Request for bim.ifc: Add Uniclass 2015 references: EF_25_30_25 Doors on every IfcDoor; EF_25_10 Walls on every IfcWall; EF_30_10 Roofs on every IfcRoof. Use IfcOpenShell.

First a look at what the model holds.

```python
import ifcopenshell

model = ifcopenshell.open("bim.ifc")
print(model.schema)
print("classifications:", [c.Name for c in model.by_type("IfcClassification")])
for ifc_class in ("IfcDoor", "IfcRoof", "IfcStair", "IfcWall", "IfcWindow"):
    print(ifc_class, len(model.by_type(ifc_class)))
```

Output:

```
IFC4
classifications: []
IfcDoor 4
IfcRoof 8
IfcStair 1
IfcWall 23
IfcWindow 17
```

```python
import ifcopenshell
import ifcopenshell.api.classification

model = ifcopenshell.open("bim.ifc")

system = ifcopenshell.api.classification.add_classification(model, classification="Uniclass 2015")

codes = {
    "IfcDoor": ("EF_25_30_25", "Doors"),
    "IfcWall": ("EF_25_10", "Walls"),
    "IfcRoof": ("EF_30_10", "Roofs"),
}
for ifc_class, (code, name) in codes.items():
    products = model.by_type(ifc_class)
    ifcopenshell.api.classification.add_reference(
        model, products=products, classification=system, identification=code, name=name
    )
    print(code, len(products))

model.write("bim_updated.ifc")
```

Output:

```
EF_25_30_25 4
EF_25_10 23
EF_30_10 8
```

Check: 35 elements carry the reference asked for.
